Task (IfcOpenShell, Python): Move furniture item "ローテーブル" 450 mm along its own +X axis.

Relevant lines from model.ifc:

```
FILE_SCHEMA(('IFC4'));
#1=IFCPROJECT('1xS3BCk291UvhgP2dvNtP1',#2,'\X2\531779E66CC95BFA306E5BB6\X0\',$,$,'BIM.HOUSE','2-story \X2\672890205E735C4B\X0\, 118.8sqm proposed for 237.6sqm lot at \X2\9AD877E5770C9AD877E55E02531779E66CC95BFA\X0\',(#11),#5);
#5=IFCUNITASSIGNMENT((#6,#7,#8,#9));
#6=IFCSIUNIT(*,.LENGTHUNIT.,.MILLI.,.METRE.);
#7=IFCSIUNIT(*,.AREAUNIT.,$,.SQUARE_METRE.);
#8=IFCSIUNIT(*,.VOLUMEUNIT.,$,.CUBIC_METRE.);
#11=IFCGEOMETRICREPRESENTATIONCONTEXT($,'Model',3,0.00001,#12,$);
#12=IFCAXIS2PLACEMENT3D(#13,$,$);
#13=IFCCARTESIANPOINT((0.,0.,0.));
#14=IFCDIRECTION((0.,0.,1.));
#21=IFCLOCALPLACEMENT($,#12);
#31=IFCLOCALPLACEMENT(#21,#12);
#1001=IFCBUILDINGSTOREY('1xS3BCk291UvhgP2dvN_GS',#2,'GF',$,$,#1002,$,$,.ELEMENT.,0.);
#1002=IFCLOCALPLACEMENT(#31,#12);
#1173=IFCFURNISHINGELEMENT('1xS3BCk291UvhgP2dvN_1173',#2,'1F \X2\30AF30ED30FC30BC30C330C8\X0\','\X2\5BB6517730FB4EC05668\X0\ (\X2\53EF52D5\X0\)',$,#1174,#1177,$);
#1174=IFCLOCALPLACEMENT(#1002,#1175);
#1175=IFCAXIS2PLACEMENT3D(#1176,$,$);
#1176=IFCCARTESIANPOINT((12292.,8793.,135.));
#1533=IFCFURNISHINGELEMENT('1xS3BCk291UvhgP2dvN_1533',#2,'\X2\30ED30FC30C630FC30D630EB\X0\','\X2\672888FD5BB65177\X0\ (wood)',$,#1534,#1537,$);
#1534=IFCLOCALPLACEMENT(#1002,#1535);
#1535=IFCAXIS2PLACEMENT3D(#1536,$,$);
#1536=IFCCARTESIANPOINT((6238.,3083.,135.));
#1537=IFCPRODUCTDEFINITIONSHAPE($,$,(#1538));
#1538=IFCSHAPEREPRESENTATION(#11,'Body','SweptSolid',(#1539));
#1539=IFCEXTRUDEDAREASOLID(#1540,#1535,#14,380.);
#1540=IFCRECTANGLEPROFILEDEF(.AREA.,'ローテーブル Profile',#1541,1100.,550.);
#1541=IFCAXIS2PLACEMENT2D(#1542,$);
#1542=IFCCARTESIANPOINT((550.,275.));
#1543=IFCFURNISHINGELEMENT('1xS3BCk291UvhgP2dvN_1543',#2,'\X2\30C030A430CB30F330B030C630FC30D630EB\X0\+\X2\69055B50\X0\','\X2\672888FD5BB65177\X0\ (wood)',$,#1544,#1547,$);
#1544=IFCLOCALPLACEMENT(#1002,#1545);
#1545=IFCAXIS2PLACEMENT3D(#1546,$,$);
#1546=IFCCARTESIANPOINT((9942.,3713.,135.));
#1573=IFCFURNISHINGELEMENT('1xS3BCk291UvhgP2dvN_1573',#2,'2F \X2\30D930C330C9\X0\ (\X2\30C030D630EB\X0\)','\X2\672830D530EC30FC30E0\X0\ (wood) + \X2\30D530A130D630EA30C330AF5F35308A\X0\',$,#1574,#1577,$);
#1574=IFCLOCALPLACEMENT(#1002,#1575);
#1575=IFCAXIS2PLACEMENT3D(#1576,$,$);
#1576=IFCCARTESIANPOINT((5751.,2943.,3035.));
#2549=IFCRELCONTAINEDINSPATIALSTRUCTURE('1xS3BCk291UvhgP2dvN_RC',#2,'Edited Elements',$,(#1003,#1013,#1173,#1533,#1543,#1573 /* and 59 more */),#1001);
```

```python
import ifcopenshell
import ifcopenshell.api.geometry
import ifcopenshell.util.placement
import ifcopenshell.util.unit

model = ifcopenshell.open("model.ifc")
unit_scale = ifcopenshell.util.unit.calculate_unit_scale(model)

item = model.by_guid("1xS3BCk291UvhgP2dvN_1533")
matrix = ifcopenshell.util.placement.get_local_placement(item.ObjectPlacement)
matrix[:3, 3] += matrix[:3, 0] * 0.45 / unit_scale
ifcopenshell.api.geometry.edit_object_placement(model, product=item, matrix=matrix, is_si=False)

print(ifcopenshell.util.placement.get_local_placement(item.ObjectPlacement).round(3) + 0.0)

model.write("model_edited.ifc")
```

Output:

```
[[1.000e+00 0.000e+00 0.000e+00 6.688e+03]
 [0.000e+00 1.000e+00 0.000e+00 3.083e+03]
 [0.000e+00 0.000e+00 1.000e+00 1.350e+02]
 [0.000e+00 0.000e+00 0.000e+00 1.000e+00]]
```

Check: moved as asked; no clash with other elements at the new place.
